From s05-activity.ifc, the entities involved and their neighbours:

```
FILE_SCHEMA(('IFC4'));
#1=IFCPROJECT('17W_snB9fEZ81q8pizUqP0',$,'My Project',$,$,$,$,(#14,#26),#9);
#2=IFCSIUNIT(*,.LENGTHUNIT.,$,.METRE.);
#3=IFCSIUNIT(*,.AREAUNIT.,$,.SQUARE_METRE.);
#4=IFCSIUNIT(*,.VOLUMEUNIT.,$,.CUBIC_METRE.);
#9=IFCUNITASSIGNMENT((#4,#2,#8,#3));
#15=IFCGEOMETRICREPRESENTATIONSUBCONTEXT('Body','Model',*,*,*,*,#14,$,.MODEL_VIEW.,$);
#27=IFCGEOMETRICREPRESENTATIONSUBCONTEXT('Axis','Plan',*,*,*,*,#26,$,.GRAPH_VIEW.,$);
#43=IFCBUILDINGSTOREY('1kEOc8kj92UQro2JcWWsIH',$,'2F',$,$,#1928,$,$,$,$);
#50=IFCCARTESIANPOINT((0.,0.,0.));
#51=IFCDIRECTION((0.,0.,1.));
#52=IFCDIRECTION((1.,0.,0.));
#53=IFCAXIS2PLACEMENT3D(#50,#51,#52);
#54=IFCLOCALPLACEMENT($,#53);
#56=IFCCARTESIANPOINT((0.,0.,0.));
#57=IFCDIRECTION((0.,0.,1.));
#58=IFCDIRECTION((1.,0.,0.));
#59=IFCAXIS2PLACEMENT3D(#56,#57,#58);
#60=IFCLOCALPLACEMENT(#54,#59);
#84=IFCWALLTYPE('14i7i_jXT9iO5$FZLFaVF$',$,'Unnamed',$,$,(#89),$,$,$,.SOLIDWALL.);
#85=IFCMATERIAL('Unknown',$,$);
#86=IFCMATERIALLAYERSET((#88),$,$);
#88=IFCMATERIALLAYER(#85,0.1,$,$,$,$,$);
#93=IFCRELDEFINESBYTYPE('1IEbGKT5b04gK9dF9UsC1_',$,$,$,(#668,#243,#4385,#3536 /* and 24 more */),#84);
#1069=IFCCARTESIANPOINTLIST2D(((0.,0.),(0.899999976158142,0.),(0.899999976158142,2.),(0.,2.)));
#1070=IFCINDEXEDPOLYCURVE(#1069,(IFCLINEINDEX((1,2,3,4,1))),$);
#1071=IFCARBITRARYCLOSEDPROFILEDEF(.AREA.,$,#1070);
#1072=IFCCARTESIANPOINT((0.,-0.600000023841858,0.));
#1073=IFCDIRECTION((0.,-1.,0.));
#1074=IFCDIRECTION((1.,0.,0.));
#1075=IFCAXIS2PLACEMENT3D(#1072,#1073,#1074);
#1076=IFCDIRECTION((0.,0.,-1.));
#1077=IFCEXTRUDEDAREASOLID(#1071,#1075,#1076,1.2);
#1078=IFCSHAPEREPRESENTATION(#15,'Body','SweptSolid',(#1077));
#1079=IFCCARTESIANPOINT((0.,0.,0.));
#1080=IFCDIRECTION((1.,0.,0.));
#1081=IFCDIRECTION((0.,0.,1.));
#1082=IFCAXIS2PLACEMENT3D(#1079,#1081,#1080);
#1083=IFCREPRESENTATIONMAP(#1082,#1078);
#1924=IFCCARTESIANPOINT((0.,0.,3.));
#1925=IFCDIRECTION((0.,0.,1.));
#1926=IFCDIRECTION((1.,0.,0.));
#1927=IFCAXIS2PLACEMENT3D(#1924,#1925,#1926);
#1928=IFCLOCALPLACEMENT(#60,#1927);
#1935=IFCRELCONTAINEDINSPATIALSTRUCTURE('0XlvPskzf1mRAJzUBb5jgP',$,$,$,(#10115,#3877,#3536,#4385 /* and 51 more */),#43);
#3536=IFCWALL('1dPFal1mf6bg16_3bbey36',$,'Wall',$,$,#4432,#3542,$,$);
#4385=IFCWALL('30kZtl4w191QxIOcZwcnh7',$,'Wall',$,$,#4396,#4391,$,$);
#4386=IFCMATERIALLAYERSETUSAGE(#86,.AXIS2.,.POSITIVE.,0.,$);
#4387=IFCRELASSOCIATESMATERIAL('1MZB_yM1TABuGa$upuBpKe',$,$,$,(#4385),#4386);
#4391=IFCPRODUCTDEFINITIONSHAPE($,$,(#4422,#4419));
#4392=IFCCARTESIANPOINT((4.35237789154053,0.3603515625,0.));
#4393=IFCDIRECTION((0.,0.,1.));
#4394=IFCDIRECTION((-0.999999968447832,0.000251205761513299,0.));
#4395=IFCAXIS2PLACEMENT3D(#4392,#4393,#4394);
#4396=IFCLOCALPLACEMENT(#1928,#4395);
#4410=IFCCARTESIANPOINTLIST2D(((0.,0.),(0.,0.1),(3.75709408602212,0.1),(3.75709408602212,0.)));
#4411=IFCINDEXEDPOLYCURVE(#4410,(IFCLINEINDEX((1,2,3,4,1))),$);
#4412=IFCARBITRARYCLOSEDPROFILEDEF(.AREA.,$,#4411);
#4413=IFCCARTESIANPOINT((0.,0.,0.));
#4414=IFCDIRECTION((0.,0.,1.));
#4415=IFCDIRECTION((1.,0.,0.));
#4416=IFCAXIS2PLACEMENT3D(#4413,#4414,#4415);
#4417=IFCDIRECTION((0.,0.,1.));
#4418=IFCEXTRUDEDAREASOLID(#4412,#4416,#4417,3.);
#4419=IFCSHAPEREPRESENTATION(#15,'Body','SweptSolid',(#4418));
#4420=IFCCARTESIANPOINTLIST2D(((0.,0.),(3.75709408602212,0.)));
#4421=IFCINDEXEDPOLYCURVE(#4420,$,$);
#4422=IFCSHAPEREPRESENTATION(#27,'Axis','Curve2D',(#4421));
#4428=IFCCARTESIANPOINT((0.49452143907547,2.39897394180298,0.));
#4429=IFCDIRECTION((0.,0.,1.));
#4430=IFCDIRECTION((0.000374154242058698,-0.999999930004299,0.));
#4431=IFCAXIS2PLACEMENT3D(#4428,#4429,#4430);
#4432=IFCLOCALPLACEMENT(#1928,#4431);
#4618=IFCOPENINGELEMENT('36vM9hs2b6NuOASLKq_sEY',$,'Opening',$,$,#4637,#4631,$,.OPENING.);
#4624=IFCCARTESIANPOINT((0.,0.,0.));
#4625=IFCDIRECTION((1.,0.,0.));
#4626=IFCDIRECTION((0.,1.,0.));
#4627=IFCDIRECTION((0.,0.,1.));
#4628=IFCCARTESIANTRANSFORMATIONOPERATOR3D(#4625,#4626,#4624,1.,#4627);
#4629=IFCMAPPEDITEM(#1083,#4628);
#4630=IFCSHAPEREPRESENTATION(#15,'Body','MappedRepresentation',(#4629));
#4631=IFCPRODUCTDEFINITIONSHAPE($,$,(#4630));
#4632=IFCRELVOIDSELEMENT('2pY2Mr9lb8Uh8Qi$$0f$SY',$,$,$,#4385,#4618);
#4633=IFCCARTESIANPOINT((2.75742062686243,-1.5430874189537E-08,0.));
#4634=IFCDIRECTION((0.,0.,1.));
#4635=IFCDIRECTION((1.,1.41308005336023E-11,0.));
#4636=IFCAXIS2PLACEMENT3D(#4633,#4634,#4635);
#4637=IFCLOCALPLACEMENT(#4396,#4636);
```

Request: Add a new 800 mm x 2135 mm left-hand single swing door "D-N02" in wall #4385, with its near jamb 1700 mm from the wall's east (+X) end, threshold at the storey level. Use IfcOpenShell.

```python
import numpy as np
import ifcopenshell
import ifcopenshell.api.feature
import ifcopenshell.api.geometry
import ifcopenshell.api.root
import ifcopenshell.api.spatial
import ifcopenshell.geom
import ifcopenshell.util.element
import ifcopenshell.util.placement
import ifcopenshell.util.representation
import ifcopenshell.util.shape
import ifcopenshell.util.unit

model = ifcopenshell.open("s05-activity.ifc")
unit_scale = ifcopenshell.util.unit.calculate_unit_scale(model)
settings = ifcopenshell.geom.settings()


def volume(element):
    """Net volume in cubic metres, openings subtracted."""
    shape = ifcopenshell.geom.create_shape(settings, element)
    return ifcopenshell.util.shape.get_volume(shape.geometry)


wall = model.by_guid("30kZtl4w191QxIOcZwcnh7")
storey = ifcopenshell.util.element.get_container(wall, ifc_class="IfcBuildingStorey")
context = ifcopenshell.util.representation.get_context(model, "Model", "Body", "MODEL_VIEW")
before = volume(wall)

width, height, from_end, sill = 0.8, 2.135, 1.7, 0.0  # metres

# The wall runs along its own X axis, and the end named is its -X end.
wall_shape = ifcopenshell.geom.create_shape(settings, wall)
x, y, z = ifcopenshell.util.shape.get_vertices(wall_shape.geometry).T
start = x.min() + from_end
face, thickness = float(y.min()), float(y.max() - y.min())
wall_matrix = ifcopenshell.util.placement.get_local_placement(wall.ObjectPlacement)
level = ifcopenshell.util.placement.get_local_placement(storey.ObjectPlacement)[2, 3]


def in_wall(x, y):
    """Placement at x, y metres in the wall's axes, at sill height."""
    matrix = wall_matrix.copy()
    matrix[:, 3] = wall_matrix @ np.array([x / unit_scale, y / unit_scale, 0.0, 1.0])
    matrix[2, 3] = level + sill / unit_scale
    return matrix


# Opening: a box that overshoots both wall faces by 50 mm.
opening = ifcopenshell.api.root.create_entity(model, ifc_class="IfcOpeningElement", predefined_type="OPENING")
box = ifcopenshell.api.geometry.add_wall_representation(
    model, context=context, length=width, height=height, thickness=thickness + 0.1
)
ifcopenshell.api.geometry.assign_representation(model, product=opening, representation=box)
ifcopenshell.api.geometry.edit_object_placement(model, product=opening, matrix=in_wall(start, face - 0.05), is_si=False)
ifcopenshell.api.feature.add_feature(model, feature=opening, element=wall)

door = ifcopenshell.api.root.create_entity(model, ifc_class="IfcDoor", name="D-N02", predefined_type="DOOR")
door.OverallWidth, door.OverallHeight = width / unit_scale, height / unit_scale
door.OperationType = "SINGLE_SWING_LEFT"
body = ifcopenshell.api.geometry.add_door_representation(
    model,
    context=context,
    overall_width=door.OverallWidth,
    overall_height=door.OverallHeight,
    operation_type="SINGLE_SWING_LEFT",
    lining_properties={"LiningDepth": thickness / unit_scale, "ThresholdDepth": thickness / unit_scale},
)
ifcopenshell.api.geometry.assign_representation(model, product=door, representation=body)
ifcopenshell.api.spatial.assign_container(model, products=[door], relating_structure=storey)
ifcopenshell.api.feature.add_filling(model, opening=opening, element=door)

# The lining spans the wall, so the door starts at the wall face.
ifcopenshell.api.geometry.edit_object_placement(model, product=door, matrix=in_wall(start, face), is_si=False)

after = volume(wall)

print(f"wall volume {before:.3f} -> {after:.3f} m3")

model.write("s05-activity_updated.ifc")
```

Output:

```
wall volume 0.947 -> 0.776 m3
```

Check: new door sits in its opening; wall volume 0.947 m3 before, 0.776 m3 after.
